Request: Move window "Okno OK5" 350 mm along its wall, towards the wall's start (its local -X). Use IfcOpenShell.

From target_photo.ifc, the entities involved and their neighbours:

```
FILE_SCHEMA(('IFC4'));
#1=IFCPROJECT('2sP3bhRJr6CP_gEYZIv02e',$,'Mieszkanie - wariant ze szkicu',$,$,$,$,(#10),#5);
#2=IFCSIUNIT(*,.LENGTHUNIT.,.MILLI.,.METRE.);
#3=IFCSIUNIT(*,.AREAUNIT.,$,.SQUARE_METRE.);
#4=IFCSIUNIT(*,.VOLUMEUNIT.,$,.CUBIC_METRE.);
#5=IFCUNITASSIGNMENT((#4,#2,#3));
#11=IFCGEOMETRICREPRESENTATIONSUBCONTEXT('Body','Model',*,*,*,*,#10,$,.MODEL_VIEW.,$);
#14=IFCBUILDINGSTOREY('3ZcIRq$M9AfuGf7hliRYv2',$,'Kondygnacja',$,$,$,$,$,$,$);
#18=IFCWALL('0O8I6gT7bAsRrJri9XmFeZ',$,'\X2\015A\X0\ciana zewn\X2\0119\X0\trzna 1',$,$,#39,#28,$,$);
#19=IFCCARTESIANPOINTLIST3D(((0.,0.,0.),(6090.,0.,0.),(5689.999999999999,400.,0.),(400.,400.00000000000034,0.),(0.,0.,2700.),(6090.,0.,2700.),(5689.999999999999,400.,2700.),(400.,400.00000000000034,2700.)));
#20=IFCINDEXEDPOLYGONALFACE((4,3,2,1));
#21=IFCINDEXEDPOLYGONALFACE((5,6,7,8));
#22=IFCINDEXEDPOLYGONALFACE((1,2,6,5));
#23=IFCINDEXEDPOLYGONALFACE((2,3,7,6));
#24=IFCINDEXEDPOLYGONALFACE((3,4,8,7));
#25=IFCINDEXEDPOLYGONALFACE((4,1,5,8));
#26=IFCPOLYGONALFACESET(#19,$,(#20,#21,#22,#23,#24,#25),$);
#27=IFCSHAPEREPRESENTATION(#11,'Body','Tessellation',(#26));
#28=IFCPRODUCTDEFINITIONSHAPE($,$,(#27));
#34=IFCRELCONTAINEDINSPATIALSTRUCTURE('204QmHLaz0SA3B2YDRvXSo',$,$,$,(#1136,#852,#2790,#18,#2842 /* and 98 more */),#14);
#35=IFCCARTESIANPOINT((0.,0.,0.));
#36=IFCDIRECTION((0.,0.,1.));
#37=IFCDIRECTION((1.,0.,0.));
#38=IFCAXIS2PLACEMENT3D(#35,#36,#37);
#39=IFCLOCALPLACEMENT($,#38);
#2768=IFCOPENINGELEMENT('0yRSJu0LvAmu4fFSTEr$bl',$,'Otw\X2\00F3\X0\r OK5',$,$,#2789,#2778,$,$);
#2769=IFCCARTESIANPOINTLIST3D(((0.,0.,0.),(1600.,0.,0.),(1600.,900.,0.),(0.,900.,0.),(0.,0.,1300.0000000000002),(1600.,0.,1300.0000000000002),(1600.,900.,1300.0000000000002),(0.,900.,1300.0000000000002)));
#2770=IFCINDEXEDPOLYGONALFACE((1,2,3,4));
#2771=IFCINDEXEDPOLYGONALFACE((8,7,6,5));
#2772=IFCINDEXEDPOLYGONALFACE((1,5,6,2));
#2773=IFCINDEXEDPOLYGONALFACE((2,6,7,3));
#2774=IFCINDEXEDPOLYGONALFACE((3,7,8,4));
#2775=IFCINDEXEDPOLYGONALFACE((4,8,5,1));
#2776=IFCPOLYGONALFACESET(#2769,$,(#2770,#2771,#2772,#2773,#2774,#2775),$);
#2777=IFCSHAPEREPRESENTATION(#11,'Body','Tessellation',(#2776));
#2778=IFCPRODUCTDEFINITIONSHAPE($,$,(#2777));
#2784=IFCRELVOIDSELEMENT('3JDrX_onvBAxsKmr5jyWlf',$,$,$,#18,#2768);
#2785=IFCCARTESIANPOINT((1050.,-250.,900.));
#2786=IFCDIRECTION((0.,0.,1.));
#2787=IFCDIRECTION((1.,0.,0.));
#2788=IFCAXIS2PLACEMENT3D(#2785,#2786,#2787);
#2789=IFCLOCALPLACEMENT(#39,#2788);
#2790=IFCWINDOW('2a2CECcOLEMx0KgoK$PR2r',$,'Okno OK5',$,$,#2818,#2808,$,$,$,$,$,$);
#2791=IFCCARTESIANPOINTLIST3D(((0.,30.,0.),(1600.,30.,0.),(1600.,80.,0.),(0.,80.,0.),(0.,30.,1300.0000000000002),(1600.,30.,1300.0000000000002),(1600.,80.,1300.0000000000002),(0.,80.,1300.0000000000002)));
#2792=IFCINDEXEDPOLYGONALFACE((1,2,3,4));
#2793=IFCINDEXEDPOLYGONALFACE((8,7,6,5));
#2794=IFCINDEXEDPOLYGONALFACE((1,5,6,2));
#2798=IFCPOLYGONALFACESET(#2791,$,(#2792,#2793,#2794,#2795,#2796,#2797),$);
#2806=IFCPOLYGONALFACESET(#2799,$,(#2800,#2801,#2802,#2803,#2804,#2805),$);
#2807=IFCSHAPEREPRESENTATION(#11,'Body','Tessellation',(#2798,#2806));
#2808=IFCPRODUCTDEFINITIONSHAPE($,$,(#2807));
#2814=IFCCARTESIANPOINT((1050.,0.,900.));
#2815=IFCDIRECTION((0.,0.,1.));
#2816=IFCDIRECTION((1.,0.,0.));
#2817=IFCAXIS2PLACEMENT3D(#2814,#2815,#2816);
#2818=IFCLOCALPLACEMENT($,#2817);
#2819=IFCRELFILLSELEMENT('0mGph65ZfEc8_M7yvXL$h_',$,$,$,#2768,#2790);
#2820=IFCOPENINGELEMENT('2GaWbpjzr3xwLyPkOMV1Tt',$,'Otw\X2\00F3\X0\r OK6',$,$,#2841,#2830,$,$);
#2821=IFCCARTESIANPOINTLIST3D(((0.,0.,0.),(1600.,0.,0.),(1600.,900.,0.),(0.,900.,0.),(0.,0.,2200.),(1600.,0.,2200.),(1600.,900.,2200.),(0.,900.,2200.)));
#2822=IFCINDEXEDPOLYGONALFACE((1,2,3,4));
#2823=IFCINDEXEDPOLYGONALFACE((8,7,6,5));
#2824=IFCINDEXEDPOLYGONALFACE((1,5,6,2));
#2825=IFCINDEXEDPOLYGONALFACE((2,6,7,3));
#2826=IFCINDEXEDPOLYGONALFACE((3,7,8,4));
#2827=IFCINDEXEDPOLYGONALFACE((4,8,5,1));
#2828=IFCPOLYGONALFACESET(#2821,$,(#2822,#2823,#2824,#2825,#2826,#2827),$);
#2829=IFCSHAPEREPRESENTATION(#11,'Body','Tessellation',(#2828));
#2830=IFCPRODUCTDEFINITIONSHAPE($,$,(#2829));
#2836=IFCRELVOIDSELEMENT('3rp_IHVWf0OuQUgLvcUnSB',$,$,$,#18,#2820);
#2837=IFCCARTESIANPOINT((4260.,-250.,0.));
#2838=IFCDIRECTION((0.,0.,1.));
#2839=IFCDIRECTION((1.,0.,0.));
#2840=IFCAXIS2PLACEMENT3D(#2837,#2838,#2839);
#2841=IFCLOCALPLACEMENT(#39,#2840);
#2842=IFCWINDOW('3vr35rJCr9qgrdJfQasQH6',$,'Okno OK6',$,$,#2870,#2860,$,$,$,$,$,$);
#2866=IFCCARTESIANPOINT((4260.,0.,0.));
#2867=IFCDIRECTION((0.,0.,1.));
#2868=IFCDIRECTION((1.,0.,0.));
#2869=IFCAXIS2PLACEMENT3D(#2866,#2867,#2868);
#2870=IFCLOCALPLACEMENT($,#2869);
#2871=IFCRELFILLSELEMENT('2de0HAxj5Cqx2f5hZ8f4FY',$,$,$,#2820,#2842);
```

```python
import ifcopenshell
import ifcopenshell.api.geometry
import ifcopenshell.util.placement
import ifcopenshell.util.unit

model = ifcopenshell.open("target_photo.ifc")
unit_scale = ifcopenshell.util.unit.calculate_unit_scale(model)

window = model.by_guid("2a2CECcOLEMx0KgoK$PR2r")
opening = window.FillsVoids[0].RelatingOpeningElement
wall = opening.VoidsElements[0].RelatingBuildingElement

wall_matrix = ifcopenshell.util.placement.get_local_placement(wall.ObjectPlacement)
shift = wall_matrix[:3, 0] * -0.35 / unit_scale
before = ifcopenshell.util.placement.get_local_placement(window.ObjectPlacement)[:3, 3].copy()

# The window is not placed relative to its opening, so move both.
for product in (opening, window):
    matrix = ifcopenshell.util.placement.get_local_placement(product.ObjectPlacement)
    matrix[:3, 3] += shift
    ifcopenshell.api.geometry.edit_object_placement(model, product=product, matrix=matrix, is_si=False)

after = ifcopenshell.util.placement.get_local_placement(window.ObjectPlacement)[:3, 3]
print("window moved by", (after - before).round(3) + 0.0)

model.write("target_photo-out.ifc")
```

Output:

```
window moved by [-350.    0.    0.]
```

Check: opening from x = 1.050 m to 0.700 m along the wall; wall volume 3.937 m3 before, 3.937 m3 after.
